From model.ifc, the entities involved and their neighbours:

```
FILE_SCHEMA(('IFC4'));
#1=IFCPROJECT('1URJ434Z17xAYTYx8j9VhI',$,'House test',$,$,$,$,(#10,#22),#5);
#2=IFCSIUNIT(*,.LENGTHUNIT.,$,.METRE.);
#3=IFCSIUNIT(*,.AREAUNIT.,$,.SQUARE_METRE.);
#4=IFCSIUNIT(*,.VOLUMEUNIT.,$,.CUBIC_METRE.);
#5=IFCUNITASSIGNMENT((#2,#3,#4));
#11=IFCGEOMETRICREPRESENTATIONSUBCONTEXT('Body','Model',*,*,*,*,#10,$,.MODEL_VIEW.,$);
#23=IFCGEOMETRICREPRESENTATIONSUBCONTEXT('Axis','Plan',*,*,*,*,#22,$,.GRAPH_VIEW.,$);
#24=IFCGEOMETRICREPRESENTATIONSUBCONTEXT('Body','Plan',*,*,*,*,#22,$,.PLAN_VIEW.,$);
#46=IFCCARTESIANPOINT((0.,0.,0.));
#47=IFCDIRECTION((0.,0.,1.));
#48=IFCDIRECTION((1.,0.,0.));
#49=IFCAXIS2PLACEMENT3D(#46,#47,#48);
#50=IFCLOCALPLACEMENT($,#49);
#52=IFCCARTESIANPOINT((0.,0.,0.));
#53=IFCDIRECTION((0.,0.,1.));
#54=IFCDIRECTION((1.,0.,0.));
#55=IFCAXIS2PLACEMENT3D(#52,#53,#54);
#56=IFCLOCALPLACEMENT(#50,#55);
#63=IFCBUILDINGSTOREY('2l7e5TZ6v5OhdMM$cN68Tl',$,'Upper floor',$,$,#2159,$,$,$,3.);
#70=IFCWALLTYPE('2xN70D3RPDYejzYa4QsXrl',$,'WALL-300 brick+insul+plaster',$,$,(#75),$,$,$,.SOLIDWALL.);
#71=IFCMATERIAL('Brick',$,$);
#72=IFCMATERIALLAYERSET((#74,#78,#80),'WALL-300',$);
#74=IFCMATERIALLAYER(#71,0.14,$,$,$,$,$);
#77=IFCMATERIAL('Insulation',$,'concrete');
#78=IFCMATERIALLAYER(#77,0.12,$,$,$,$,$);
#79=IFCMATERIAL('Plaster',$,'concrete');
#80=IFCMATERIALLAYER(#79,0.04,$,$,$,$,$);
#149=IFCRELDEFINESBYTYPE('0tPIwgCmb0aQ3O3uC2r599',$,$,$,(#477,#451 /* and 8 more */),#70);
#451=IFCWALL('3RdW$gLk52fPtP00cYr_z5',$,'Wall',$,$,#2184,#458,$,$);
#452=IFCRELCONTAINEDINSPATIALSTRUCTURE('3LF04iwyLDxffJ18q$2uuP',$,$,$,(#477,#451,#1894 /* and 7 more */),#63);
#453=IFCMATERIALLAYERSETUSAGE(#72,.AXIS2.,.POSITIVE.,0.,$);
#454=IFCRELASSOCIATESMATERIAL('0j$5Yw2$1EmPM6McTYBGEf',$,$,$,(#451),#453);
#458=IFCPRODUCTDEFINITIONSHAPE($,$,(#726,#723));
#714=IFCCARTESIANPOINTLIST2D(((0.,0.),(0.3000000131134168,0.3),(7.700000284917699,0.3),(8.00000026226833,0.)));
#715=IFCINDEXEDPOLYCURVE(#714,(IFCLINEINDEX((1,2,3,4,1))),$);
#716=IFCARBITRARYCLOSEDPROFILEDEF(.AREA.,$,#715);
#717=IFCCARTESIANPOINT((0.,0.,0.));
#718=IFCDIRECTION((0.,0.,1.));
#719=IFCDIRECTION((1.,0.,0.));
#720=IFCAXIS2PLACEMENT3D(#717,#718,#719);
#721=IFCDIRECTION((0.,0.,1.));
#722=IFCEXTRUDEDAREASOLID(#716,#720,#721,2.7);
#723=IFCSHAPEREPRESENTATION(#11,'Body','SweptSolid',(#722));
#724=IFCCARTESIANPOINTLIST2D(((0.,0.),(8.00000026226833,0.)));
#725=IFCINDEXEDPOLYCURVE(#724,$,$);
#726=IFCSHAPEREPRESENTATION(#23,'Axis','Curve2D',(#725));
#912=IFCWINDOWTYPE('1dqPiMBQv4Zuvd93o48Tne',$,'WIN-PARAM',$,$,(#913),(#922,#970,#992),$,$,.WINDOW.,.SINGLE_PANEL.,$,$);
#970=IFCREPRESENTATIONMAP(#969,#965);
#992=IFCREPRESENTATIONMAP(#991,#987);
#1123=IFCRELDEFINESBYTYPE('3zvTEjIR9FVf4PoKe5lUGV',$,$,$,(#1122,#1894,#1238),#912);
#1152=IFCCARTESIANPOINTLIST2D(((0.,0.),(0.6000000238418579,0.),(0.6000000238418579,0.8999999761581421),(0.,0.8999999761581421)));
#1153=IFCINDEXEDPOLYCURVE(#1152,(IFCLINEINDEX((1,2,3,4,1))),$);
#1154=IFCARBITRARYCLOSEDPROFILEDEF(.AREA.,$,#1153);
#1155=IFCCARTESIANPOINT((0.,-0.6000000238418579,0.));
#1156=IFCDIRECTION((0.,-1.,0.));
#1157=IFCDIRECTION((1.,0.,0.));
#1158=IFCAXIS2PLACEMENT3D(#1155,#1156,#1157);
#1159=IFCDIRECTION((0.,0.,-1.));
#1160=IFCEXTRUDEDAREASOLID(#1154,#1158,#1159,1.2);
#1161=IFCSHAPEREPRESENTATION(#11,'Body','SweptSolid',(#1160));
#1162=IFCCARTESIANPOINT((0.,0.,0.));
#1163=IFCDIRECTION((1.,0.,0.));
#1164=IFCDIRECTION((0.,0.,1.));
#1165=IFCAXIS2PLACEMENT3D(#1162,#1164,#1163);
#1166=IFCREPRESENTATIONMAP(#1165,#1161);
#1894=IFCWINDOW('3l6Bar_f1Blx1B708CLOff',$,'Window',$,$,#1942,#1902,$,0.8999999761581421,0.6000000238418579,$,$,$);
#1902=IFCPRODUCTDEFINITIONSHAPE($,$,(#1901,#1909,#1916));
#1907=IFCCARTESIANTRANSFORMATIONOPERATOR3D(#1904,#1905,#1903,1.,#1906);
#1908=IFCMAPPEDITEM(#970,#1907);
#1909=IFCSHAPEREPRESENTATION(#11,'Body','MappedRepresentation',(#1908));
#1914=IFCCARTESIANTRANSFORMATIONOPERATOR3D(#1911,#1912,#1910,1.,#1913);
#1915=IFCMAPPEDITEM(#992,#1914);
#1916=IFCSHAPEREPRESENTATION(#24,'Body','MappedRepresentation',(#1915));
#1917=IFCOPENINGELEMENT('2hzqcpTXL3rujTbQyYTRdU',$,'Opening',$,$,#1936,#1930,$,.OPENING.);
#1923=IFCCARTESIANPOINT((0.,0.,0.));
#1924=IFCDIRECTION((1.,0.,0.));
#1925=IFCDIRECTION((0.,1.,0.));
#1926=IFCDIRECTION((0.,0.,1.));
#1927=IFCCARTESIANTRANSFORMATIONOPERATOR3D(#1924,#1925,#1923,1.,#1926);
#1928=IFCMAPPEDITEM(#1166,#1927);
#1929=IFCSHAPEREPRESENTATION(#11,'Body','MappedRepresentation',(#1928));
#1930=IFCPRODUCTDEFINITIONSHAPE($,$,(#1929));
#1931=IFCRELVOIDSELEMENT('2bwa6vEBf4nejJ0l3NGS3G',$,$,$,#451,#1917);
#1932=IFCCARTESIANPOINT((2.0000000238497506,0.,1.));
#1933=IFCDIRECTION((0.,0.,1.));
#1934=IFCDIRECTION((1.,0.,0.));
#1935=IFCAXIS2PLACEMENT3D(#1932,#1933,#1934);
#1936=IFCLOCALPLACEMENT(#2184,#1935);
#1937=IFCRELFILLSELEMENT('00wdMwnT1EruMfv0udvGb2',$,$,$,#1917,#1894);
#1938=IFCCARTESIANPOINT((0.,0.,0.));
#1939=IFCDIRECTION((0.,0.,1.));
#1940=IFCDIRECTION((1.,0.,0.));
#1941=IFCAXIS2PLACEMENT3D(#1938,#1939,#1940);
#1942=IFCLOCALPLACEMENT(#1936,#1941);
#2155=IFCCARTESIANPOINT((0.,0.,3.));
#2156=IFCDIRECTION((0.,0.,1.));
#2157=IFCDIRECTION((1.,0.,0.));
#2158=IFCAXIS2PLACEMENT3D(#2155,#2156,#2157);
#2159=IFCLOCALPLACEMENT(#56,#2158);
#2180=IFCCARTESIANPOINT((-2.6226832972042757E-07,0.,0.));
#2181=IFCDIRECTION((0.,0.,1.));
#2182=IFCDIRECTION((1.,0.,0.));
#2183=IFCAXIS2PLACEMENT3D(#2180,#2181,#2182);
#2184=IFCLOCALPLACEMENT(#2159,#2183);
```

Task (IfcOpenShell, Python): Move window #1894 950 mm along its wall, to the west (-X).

```python
import ifcopenshell
import ifcopenshell.api.geometry
import ifcopenshell.util.placement

model = ifcopenshell.open("model.ifc")

window = model.by_id(1894)
opening = window.FillsVoids[0].RelatingOpeningElement
wall = opening.VoidsElements[0].RelatingBuildingElement

wall_matrix = ifcopenshell.util.placement.get_local_placement(wall.ObjectPlacement)
shift = wall_matrix[:3, 0] * -0.95
before = ifcopenshell.util.placement.get_local_placement(window.ObjectPlacement)[:3, 3].copy()

# The window is placed relative to its opening, so it follows when the opening moves.
matrix = ifcopenshell.util.placement.get_local_placement(opening.ObjectPlacement)
matrix[:3, 3] += shift
ifcopenshell.api.geometry.edit_object_placement(
    model, product=opening, matrix=matrix, is_si=False, should_transform_children=True
)

after = ifcopenshell.util.placement.get_local_placement(window.ObjectPlacement)[:3, 3]
print("window moved by", (after - before).round(3) + 0.0)

model.write("model-out.ifc")
```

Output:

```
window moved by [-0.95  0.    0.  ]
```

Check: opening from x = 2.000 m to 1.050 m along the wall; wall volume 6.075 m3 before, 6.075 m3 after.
